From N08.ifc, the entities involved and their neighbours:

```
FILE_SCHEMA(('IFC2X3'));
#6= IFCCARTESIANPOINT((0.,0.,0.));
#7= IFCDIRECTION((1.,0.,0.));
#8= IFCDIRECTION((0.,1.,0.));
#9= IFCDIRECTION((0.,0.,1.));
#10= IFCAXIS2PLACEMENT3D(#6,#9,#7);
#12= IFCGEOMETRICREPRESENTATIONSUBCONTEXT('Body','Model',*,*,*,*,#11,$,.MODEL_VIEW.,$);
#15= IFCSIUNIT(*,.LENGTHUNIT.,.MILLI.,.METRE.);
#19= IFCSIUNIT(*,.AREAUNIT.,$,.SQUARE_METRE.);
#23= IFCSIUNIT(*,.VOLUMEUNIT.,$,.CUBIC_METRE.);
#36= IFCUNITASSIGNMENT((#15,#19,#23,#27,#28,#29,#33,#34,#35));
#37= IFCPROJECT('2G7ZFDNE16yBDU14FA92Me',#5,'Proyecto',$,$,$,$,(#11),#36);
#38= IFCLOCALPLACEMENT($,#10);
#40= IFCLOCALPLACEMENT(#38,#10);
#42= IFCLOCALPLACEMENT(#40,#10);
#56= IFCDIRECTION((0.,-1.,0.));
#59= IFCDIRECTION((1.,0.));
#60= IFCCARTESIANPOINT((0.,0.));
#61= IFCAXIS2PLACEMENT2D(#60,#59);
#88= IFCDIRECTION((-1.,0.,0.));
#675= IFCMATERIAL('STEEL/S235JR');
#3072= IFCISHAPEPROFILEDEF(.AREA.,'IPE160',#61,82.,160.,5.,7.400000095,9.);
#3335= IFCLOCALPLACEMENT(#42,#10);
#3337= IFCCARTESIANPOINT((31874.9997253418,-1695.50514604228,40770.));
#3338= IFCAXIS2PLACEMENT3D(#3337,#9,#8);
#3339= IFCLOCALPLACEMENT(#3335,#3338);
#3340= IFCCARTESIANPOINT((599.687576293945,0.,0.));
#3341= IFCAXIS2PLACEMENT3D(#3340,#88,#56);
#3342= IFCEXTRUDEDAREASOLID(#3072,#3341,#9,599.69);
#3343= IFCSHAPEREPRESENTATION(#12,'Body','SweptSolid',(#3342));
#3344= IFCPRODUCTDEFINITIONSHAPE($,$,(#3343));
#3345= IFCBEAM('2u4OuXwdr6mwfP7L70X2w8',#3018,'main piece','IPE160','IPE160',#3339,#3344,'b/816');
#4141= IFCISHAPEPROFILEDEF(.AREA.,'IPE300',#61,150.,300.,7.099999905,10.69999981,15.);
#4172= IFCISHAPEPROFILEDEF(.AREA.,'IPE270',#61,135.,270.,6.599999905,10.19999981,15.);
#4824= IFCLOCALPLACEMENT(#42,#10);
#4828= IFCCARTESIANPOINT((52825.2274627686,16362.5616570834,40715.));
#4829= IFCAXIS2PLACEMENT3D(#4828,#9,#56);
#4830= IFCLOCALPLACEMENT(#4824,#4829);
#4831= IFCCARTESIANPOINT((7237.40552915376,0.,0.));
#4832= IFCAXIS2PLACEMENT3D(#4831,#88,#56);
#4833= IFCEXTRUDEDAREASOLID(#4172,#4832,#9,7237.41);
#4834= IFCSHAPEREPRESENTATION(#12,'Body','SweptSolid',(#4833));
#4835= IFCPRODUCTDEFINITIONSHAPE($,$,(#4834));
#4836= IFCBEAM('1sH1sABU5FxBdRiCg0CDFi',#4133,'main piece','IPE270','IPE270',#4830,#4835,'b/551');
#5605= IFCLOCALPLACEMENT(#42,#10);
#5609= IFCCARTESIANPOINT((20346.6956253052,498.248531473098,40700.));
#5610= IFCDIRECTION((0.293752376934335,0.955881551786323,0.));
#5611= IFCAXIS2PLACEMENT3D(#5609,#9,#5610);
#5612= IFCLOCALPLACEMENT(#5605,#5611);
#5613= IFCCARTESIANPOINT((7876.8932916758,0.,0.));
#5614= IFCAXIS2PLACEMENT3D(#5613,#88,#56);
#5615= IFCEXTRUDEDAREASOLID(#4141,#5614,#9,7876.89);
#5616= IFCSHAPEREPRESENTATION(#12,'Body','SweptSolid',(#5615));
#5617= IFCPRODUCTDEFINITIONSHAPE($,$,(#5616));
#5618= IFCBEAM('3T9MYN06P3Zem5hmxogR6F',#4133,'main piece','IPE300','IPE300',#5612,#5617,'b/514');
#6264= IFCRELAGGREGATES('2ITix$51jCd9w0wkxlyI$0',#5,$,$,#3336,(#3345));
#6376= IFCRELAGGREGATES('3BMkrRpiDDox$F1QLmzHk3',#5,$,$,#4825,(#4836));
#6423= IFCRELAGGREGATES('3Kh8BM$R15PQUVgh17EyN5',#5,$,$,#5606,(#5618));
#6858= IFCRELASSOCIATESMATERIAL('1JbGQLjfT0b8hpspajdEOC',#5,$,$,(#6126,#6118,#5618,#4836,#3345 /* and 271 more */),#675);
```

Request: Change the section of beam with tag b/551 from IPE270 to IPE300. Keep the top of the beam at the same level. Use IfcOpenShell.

```python
import ifcopenshell
import ifcopenshell.util.element
import ifcopenshell.util.representation

model = ifcopenshell.open("N08.ifc")

member = model.by_id(4836)
source = next(p for p in model.by_type("IfcIShapeProfileDef") if p.ProfileName == "IPE300")

body = ifcopenshell.util.representation.get_representation(member, "Model", "Body")
solid = body.Items[0]
old_profile = solid.SweptArea

# Copy the section's sizes but keep this member's own profile position.
profile = ifcopenshell.util.element.copy(model, source)
# Profiles are centred, so shift by half the change in depth to hold the top.
shift = (old_profile.OverallDepth - profile.OverallDepth) / 2
x, y = old_profile.Position.Location.Coordinates
up = (0.0, 1.0)  # upwards, in the solid's own plane
location = model.createIfcCartesianPoint((x + up[0] * shift, y + up[1] * shift))
profile.Position = model.createIfcAxis2Placement2D(location, old_profile.Position.RefDirection)
solid.SweptArea = profile
if not model.get_total_inverses(old_profile):
    ifcopenshell.util.element.remove_deep2(model, old_profile)
member.Description = member.Description.replace("IPE270", "IPE300")
member.ObjectType = member.ObjectType.replace("IPE270", "IPE300")

print(solid.SweptArea)

model.write("N08_edited.ifc")
```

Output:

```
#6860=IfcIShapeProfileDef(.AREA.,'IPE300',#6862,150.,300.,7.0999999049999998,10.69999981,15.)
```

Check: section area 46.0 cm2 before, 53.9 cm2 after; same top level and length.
